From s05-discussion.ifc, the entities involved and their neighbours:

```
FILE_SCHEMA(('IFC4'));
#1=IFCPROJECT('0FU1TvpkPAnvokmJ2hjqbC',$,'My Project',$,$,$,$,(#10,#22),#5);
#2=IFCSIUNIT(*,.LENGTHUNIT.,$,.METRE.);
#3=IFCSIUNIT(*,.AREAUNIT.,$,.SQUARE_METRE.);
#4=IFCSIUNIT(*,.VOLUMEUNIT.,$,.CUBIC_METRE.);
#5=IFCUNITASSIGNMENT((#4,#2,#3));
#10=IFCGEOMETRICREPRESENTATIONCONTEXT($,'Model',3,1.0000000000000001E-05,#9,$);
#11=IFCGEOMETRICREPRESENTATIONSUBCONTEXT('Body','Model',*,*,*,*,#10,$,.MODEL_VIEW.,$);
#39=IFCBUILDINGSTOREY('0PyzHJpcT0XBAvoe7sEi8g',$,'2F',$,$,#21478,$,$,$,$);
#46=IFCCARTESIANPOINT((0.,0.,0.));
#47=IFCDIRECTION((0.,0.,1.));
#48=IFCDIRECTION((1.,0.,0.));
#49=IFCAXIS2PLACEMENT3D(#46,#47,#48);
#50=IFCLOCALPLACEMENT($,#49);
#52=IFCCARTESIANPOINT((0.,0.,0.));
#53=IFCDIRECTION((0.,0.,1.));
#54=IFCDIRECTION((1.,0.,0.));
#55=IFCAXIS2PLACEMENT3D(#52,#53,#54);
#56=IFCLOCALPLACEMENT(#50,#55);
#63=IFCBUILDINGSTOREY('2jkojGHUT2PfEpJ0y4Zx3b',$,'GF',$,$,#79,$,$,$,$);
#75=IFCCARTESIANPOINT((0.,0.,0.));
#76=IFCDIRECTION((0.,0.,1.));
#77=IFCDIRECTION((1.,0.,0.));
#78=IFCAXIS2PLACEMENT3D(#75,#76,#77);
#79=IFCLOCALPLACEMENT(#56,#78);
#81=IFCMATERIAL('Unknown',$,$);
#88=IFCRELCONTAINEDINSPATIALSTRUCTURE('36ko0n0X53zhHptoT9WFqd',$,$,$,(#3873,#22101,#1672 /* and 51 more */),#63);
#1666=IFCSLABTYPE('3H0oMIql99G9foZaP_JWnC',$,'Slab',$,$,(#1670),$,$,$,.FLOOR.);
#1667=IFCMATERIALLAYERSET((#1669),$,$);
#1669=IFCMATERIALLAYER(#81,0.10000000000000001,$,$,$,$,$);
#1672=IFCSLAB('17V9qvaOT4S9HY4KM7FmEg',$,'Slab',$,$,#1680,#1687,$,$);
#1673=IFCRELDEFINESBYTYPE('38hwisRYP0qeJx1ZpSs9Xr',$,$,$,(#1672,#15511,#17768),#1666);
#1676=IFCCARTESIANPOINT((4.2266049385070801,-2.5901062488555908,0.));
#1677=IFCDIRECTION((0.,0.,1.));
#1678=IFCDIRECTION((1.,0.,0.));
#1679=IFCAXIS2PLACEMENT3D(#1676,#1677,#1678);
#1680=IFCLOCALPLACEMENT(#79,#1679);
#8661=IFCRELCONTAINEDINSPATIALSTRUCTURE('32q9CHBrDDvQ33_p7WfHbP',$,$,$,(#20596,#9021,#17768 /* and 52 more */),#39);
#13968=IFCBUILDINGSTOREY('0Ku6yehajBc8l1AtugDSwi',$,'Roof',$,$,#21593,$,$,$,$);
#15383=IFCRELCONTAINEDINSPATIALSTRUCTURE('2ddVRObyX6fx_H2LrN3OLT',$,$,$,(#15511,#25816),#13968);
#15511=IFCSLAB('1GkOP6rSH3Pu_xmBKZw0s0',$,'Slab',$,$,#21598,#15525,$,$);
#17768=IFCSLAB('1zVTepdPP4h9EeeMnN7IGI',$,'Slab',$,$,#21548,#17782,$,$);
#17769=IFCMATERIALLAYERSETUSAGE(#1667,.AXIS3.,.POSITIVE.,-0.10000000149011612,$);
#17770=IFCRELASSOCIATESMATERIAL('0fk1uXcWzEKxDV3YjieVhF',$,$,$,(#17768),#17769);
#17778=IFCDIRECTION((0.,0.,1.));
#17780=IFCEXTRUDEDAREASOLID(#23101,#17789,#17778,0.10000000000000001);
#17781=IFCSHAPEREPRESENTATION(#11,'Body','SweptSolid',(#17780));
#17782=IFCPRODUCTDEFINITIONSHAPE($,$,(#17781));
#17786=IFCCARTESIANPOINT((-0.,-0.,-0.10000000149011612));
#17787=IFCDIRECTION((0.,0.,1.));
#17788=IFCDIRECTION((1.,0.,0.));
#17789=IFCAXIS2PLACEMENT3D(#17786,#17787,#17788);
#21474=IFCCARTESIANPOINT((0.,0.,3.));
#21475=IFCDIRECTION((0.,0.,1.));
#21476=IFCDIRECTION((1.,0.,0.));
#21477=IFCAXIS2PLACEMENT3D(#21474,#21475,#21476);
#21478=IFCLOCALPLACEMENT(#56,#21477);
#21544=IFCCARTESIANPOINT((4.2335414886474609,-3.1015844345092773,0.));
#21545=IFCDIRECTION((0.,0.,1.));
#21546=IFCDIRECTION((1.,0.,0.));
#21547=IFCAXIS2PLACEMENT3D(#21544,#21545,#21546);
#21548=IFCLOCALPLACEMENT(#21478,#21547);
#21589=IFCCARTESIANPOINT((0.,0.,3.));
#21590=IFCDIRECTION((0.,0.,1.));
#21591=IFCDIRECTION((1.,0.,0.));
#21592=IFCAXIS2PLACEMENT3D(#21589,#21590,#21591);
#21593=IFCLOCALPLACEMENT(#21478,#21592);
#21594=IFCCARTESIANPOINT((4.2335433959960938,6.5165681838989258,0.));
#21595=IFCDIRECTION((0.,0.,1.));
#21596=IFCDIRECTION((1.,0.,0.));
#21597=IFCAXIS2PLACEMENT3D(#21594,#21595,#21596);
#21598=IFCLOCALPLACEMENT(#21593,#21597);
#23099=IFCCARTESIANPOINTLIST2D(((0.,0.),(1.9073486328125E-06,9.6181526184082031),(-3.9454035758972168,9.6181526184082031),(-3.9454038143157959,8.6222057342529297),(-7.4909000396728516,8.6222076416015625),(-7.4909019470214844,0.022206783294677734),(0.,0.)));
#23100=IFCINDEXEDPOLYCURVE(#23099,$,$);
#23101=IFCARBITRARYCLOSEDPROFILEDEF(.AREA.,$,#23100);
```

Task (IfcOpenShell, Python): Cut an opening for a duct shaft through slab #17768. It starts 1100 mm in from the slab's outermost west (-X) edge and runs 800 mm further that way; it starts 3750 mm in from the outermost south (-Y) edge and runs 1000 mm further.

```python
import numpy as np
import ifcopenshell
import ifcopenshell.api.feature
import ifcopenshell.api.geometry
import ifcopenshell.api.root
import ifcopenshell.geom
import ifcopenshell.util.placement
import ifcopenshell.util.representation
import ifcopenshell.util.shape
import ifcopenshell.util.unit

model = ifcopenshell.open("s05-discussion.ifc")
unit_scale = ifcopenshell.util.unit.calculate_unit_scale(model)
settings = ifcopenshell.geom.settings()


def volume(element):
    """Net volume in cubic metres, openings subtracted."""
    shape = ifcopenshell.geom.create_shape(settings, element)
    return ifcopenshell.util.shape.get_volume(shape.geometry)


slab = model.by_id(17768)
before = volume(slab)

# Extent in the slab's own axes, in metres. The edges named are its -X and -Y sides.
slab_shape = ifcopenshell.geom.create_shape(settings, slab)
vertices = ifcopenshell.util.shape.get_vertices(slab_shape.geometry)
x_min, y_min, bottom = vertices.min(axis=0)
top = vertices[:, 2].max()

opening = ifcopenshell.api.root.create_entity(model, ifc_class="IfcOpeningElement", name="Duct shaft opening", predefined_type="OPENING")
context = ifcopenshell.util.representation.get_context(model, "Model", "Body", "MODEL_VIEW")
width, depth = 0.8, 1
outline = [(0.0, 0.0), (width, 0.0), (width, depth), (0.0, depth), (0.0, 0.0)]
# Overshoot both faces by 50 mm so the cut is clean.
shape = ifcopenshell.api.geometry.add_slab_representation(
    model, context=context, depth=top - bottom + 0.1, polyline=outline
)
ifcopenshell.api.geometry.assign_representation(model, product=opening, representation=shape)

matrix = ifcopenshell.util.placement.get_local_placement(slab.ObjectPlacement)
matrix[:, 3] = matrix @ np.append(np.array([x_min + 1.1, y_min + 3.75, bottom - 0.05]) / unit_scale, 1.0)
ifcopenshell.api.geometry.edit_object_placement(model, product=opening, matrix=matrix, is_si=False)
ifcopenshell.api.feature.add_feature(model, feature=opening, element=slab)

after = volume(slab)

print(f"slab volume {before:.3f} -> {after:.3f} m3")

model.write("s05-discussion_v2.ifc")
```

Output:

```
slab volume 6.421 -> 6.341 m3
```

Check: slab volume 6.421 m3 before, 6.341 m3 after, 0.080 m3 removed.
